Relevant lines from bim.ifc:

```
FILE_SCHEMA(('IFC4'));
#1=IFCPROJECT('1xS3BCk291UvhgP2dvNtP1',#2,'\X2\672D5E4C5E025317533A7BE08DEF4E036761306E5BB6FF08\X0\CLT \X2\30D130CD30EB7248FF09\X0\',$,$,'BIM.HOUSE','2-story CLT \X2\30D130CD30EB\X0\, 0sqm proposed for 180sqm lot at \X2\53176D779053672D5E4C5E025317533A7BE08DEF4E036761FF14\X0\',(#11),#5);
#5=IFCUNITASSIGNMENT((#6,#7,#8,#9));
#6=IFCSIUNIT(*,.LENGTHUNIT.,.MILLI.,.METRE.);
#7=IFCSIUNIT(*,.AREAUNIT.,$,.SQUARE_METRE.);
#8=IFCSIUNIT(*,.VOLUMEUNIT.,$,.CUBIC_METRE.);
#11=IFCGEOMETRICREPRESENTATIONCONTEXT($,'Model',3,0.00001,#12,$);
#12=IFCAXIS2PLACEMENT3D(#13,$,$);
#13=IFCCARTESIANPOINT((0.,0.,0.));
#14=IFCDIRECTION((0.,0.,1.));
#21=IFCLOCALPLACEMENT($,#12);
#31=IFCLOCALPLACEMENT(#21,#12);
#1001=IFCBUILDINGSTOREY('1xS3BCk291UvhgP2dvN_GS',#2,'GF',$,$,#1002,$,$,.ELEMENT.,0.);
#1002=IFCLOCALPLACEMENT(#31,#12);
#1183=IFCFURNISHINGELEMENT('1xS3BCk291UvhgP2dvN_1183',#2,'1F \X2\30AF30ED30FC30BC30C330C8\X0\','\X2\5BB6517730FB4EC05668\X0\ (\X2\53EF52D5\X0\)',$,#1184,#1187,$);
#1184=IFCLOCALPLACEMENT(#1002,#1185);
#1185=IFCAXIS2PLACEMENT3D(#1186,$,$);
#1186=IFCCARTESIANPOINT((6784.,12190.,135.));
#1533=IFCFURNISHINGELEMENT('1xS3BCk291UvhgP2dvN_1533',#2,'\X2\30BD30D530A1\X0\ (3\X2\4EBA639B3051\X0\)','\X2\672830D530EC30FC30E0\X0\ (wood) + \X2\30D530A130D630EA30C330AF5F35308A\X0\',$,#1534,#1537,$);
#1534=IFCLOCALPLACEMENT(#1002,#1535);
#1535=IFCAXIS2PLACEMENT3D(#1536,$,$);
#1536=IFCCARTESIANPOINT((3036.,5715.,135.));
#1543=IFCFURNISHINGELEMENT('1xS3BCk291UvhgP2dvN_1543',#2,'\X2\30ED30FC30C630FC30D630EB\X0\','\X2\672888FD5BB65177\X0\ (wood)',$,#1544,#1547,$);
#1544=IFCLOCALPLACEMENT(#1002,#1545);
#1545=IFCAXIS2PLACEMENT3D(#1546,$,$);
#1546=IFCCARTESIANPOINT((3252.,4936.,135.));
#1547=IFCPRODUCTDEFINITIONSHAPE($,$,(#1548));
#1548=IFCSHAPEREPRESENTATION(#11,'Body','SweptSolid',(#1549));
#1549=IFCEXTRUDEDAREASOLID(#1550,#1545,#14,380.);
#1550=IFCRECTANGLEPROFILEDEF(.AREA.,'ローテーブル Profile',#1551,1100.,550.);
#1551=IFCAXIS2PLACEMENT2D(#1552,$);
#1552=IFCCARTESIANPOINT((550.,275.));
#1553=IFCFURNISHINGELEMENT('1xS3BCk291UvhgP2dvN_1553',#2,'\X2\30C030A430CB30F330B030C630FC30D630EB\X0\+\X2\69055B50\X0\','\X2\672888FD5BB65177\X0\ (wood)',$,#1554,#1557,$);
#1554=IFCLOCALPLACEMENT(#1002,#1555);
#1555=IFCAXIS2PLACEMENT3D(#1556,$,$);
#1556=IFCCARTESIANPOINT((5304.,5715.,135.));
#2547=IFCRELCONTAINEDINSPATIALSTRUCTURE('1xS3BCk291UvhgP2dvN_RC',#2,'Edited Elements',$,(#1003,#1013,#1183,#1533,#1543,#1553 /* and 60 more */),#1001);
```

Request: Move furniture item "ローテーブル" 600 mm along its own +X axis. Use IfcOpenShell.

```python
import ifcopenshell
import ifcopenshell.api.geometry
import ifcopenshell.util.placement
import ifcopenshell.util.unit

model = ifcopenshell.open("bim.ifc")
unit_scale = ifcopenshell.util.unit.calculate_unit_scale(model)

item = model.by_guid("1xS3BCk291UvhgP2dvN_1543")
matrix = ifcopenshell.util.placement.get_local_placement(item.ObjectPlacement)
matrix[:3, 3] += matrix[:3, 0] * 0.6 / unit_scale
ifcopenshell.api.geometry.edit_object_placement(model, product=item, matrix=matrix, is_si=False)

print(ifcopenshell.util.placement.get_local_placement(item.ObjectPlacement).round(3) + 0.0)

model.write("bim_v2.ifc")
```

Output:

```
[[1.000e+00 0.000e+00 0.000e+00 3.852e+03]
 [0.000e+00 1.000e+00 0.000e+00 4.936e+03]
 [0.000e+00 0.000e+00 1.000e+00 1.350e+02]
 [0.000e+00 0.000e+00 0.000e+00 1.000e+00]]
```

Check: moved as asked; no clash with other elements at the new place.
